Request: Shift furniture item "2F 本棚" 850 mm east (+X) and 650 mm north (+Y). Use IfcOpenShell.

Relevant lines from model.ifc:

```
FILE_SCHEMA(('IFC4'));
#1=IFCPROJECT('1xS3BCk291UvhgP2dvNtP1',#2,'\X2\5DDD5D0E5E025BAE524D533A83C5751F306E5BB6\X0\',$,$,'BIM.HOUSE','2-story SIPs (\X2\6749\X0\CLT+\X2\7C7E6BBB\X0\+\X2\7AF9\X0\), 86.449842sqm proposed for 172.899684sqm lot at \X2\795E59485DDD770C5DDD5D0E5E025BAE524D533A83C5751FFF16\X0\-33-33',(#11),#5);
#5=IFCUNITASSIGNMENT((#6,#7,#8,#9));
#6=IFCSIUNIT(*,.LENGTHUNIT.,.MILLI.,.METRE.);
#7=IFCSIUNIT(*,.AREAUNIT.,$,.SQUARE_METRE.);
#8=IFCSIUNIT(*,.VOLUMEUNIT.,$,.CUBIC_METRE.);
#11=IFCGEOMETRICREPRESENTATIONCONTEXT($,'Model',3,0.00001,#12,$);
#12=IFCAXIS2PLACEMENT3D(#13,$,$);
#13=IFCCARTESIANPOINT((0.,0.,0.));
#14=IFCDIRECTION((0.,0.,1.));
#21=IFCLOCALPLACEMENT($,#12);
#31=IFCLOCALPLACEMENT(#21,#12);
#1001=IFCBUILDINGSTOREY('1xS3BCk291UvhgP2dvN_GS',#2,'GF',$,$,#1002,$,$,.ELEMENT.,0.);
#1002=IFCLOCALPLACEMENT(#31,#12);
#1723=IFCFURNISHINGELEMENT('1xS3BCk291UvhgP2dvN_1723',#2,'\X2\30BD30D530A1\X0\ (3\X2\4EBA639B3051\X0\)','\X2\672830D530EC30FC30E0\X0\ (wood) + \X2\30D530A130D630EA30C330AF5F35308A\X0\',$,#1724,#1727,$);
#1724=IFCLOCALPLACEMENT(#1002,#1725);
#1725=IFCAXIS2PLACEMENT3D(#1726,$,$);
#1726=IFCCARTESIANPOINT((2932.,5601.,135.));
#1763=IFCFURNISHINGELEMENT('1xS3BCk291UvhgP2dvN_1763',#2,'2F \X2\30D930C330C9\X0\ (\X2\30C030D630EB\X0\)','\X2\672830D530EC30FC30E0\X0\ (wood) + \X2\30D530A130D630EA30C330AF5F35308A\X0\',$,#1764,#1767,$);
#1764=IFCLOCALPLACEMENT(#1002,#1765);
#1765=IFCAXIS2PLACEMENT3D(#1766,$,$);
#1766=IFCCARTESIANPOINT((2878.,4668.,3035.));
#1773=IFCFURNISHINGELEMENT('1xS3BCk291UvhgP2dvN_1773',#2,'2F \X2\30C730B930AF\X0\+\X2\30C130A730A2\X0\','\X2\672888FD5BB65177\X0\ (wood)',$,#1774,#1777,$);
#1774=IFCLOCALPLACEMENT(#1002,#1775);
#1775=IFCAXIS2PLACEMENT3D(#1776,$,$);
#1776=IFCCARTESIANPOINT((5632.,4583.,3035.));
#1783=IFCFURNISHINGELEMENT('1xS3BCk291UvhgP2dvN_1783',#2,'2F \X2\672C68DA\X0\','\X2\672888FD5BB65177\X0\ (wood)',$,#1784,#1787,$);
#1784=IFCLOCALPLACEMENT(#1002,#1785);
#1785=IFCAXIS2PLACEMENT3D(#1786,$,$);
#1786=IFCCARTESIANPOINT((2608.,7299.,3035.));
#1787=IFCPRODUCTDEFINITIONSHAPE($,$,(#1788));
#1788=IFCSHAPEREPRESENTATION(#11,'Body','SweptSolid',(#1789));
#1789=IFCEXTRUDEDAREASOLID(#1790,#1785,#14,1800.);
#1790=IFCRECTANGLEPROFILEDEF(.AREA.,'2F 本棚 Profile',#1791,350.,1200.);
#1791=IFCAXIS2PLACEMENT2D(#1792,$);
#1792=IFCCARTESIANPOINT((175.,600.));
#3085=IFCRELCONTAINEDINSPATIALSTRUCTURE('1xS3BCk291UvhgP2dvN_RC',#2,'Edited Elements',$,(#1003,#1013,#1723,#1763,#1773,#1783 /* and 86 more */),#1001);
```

```python
import ifcopenshell
import ifcopenshell.api.geometry
import ifcopenshell.util.placement
import ifcopenshell.util.unit

model = ifcopenshell.open("model.ifc")
unit_scale = ifcopenshell.util.unit.calculate_unit_scale(model)

item = model.by_guid("1xS3BCk291UvhgP2dvN_1783")
matrix = ifcopenshell.util.placement.get_local_placement(item.ObjectPlacement)
matrix[0, 3] += 0.85 / unit_scale
matrix[1, 3] += 0.65 / unit_scale
ifcopenshell.api.geometry.edit_object_placement(model, product=item, matrix=matrix, is_si=False)

print(ifcopenshell.util.placement.get_local_placement(item.ObjectPlacement).round(3) + 0.0)

model.write("model_edited.ifc")
```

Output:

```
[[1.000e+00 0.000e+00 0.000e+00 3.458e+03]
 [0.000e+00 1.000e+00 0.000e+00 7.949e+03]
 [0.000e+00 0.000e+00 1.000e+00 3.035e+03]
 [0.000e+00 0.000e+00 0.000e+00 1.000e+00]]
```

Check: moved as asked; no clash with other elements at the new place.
